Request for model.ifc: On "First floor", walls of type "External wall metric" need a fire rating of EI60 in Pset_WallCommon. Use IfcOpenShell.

First a look at what the model holds.

```python
import ifcopenshell
import ifcopenshell.util.element

model = ifcopenshell.open("model.ifc")
print(model.schema)
storey = next(s for s in model.by_type("IfcBuildingStorey") if s.Name == "First floor")
walls = [e for e in ifcopenshell.util.element.get_decomposition(storey) if e.is_a("IfcWall")]
seen = {}
for e in walls:
    element_type = ifcopenshell.util.element.get_type(e)
    key = (element_type.Name if element_type != e and element_type else None, ifcopenshell.util.element.get_pset(e, "Pset_WallCommon", "FireRating"))
    seen[key] = seen.get(key, 0) + 1
for (name, value), count in sorted(seen.items(), key=str):
    print(count, "x", name, "|", value)
```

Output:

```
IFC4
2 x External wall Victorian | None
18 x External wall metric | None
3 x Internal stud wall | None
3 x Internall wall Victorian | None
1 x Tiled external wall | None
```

```python
import ifcopenshell
import ifcopenshell.api.pset
import ifcopenshell.util.element

model = ifcopenshell.open("model.ifc")

storey = next(s for s in model.by_type("IfcBuildingStorey") if s.Name == "First floor")
walls = [e for e in ifcopenshell.util.element.get_decomposition(storey) if e.is_a("IfcWall")]

count = 0
for e in walls:
    element_type = ifcopenshell.util.element.get_type(e)
    if element_type in (None, e) or element_type.Name != "External wall metric":
        continue
    # add_pset returns the element's existing set when there is one.
    pset = ifcopenshell.api.pset.add_pset(model, product=e, name="Pset_WallCommon")
    ifcopenshell.api.pset.edit_pset(model, pset=pset, properties={"FireRating": "EI60"})
    count += 1

print(count, "walls updated")

model.write("model-out.ifc")
```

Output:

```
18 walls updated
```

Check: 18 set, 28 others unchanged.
